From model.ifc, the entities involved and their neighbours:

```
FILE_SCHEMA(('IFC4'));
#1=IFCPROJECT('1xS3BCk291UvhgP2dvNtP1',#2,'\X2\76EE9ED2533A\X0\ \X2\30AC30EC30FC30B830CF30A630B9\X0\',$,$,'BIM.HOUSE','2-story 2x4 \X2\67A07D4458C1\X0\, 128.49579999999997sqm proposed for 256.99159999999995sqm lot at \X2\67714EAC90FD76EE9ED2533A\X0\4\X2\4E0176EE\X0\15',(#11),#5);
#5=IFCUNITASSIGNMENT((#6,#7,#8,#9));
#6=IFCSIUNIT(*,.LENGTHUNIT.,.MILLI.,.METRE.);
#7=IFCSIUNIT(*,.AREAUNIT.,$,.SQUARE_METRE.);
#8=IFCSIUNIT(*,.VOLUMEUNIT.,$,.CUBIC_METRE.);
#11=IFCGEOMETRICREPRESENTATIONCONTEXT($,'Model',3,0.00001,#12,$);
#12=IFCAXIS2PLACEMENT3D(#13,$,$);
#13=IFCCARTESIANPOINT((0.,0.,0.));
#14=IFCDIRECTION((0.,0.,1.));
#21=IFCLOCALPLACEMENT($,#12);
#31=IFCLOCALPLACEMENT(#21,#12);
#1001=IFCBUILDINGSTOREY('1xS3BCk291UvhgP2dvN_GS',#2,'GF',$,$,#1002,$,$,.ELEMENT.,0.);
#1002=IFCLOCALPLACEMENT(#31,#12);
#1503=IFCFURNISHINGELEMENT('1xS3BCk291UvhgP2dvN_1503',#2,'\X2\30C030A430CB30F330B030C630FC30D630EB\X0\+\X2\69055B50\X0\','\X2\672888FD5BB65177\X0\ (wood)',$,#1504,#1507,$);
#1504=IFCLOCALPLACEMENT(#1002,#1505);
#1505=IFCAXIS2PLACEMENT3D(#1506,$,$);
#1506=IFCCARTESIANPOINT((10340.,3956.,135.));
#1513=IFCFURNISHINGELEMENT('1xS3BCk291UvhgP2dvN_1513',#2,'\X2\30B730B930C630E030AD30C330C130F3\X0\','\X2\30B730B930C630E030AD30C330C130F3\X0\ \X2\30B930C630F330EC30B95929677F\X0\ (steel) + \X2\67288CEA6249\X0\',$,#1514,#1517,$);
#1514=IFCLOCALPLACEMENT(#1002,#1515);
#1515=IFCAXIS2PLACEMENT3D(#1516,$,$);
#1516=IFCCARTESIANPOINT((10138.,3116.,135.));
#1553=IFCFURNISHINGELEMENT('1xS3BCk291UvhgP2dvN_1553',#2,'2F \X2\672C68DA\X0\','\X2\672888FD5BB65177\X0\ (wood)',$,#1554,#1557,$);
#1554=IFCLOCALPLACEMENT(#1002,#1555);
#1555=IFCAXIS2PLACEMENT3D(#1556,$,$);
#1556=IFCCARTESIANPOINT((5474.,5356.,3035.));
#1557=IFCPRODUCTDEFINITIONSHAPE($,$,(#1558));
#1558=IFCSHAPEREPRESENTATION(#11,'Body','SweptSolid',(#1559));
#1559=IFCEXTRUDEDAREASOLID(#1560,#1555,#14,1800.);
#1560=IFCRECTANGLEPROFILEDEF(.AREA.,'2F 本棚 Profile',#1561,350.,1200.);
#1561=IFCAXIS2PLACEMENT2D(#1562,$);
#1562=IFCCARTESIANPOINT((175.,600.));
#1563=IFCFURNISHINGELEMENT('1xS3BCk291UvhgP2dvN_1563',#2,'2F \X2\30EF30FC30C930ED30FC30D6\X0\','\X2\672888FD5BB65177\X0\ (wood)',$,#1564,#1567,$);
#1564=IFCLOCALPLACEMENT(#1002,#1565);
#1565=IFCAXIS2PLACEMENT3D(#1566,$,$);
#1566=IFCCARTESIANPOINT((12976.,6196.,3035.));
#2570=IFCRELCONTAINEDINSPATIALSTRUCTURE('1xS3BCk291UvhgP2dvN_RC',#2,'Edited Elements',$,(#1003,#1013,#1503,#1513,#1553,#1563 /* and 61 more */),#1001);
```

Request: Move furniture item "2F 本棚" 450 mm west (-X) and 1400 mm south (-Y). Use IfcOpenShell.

```python
import ifcopenshell
import ifcopenshell.api.geometry
import ifcopenshell.util.placement
import ifcopenshell.util.unit

model = ifcopenshell.open("model.ifc")
unit_scale = ifcopenshell.util.unit.calculate_unit_scale(model)

item = model.by_guid("1xS3BCk291UvhgP2dvN_1553")
matrix = ifcopenshell.util.placement.get_local_placement(item.ObjectPlacement)
matrix[0, 3] -= 0.45 / unit_scale
matrix[1, 3] -= 1.4 / unit_scale
ifcopenshell.api.geometry.edit_object_placement(model, product=item, matrix=matrix, is_si=False)

print(ifcopenshell.util.placement.get_local_placement(item.ObjectPlacement).round(3) + 0.0)

model.write("model_edited.ifc")
```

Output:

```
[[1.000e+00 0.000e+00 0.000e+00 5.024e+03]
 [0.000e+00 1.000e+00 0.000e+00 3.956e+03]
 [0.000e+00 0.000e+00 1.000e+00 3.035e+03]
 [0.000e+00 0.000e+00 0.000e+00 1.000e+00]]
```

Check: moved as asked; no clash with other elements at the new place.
